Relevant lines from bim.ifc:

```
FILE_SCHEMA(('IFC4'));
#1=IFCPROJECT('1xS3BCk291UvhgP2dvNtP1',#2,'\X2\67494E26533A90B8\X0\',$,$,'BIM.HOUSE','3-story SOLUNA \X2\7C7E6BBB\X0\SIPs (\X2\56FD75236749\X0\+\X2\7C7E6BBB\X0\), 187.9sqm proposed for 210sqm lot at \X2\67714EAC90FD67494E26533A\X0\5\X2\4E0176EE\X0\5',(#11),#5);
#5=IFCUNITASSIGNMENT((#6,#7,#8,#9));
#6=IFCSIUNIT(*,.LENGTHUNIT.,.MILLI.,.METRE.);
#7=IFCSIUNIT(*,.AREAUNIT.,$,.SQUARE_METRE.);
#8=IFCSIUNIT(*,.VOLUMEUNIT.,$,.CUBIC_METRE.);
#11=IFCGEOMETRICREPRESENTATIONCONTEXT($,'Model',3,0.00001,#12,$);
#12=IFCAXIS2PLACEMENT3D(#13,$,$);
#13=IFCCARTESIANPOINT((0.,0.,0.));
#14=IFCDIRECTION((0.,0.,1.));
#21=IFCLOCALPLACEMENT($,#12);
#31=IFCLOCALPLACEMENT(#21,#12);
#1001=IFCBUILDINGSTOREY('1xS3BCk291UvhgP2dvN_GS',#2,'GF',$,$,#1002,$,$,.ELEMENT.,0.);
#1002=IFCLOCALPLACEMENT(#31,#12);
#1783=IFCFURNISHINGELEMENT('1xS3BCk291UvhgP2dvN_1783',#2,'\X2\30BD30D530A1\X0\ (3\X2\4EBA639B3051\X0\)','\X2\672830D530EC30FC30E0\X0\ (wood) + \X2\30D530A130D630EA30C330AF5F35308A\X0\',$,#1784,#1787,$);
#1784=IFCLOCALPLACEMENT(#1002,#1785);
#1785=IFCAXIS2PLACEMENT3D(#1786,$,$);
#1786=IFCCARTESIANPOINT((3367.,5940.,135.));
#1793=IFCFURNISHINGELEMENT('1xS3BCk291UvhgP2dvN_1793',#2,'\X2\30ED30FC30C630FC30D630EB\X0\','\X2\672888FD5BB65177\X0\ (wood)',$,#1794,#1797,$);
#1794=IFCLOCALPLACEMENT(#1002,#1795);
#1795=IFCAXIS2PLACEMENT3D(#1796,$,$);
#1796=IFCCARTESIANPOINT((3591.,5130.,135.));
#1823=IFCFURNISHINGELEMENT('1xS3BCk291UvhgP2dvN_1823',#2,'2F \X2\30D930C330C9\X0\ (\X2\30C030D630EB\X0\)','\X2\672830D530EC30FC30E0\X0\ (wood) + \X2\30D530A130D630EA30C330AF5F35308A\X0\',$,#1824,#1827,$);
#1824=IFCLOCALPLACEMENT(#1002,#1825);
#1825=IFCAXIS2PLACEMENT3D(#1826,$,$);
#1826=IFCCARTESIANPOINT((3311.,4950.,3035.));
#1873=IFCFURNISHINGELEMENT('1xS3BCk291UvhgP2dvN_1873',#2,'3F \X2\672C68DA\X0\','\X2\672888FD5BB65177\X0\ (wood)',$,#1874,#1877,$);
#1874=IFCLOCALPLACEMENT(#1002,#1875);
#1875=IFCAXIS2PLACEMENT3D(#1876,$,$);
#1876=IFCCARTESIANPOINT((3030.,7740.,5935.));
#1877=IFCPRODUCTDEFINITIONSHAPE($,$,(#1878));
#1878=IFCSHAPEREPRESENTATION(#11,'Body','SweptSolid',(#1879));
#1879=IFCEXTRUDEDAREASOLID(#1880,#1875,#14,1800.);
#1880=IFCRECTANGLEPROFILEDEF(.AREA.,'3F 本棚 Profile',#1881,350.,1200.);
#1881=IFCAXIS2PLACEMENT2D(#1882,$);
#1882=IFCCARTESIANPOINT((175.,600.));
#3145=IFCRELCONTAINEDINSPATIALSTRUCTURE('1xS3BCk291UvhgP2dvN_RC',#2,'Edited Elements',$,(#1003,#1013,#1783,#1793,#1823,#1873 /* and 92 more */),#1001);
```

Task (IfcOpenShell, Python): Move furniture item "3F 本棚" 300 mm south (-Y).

```python
import ifcopenshell
import ifcopenshell.api.geometry
import ifcopenshell.util.placement
import ifcopenshell.util.unit

model = ifcopenshell.open("bim.ifc")
unit_scale = ifcopenshell.util.unit.calculate_unit_scale(model)

item = model.by_guid("1xS3BCk291UvhgP2dvN_1873")
matrix = ifcopenshell.util.placement.get_local_placement(item.ObjectPlacement)
matrix[1, 3] -= 0.3 / unit_scale
ifcopenshell.api.geometry.edit_object_placement(model, product=item, matrix=matrix, is_si=False)

print(ifcopenshell.util.placement.get_local_placement(item.ObjectPlacement).round(3) + 0.0)

model.write("bim_v2.ifc")
```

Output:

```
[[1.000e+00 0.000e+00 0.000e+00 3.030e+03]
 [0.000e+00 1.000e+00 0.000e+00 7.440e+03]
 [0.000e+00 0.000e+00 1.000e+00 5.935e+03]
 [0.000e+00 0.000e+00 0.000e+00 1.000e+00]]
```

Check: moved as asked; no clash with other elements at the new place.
